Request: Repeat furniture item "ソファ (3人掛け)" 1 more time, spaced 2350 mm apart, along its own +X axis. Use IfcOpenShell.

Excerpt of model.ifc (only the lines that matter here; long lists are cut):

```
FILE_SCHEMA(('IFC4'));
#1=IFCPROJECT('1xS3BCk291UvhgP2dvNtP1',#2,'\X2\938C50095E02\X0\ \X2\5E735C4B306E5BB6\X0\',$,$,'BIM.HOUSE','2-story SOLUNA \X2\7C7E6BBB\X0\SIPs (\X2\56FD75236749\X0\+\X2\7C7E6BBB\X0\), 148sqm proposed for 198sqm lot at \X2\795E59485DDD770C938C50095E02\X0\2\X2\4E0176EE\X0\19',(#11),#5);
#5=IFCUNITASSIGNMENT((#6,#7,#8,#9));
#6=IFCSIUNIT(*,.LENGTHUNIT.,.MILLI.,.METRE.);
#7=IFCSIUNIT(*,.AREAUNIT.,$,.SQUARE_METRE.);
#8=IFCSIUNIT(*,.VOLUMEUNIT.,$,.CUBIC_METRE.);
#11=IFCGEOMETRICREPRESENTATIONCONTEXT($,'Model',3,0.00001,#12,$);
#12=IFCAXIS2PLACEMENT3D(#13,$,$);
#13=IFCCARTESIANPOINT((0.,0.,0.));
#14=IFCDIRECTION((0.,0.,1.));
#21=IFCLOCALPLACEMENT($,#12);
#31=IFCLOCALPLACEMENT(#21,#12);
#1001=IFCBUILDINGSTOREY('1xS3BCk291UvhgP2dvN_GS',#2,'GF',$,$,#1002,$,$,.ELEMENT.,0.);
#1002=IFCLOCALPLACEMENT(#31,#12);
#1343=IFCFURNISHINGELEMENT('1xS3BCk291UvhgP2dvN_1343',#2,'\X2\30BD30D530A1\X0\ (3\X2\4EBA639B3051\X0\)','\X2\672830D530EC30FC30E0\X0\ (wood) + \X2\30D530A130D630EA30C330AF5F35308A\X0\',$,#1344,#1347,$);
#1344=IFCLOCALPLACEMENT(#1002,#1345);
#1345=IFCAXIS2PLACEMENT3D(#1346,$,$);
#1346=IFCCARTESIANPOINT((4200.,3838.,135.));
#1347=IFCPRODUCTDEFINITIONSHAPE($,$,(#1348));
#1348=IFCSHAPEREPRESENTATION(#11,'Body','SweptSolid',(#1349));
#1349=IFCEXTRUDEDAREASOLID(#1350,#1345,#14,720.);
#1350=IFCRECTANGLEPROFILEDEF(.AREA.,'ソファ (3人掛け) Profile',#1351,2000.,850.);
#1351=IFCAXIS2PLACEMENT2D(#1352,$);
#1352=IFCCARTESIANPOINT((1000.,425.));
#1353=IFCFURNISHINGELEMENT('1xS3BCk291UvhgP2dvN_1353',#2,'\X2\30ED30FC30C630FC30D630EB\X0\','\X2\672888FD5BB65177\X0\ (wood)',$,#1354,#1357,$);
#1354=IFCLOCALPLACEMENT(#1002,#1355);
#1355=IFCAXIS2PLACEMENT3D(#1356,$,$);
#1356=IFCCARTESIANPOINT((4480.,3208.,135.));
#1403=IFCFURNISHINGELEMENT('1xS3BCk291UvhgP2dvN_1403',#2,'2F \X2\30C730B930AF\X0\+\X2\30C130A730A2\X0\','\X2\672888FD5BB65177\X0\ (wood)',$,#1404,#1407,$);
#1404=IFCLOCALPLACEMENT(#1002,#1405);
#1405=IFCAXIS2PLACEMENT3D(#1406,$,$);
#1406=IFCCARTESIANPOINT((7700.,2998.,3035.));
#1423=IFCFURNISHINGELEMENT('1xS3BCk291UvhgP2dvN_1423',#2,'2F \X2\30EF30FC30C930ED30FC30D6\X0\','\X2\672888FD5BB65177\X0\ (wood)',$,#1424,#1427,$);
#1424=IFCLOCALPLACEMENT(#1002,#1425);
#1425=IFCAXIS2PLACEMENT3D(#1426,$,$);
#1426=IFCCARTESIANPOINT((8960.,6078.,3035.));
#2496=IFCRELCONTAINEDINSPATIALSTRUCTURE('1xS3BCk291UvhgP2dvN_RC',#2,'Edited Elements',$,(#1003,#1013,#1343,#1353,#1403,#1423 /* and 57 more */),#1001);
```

```python
import ifcopenshell
import ifcopenshell.api.geometry
import ifcopenshell.api.root
import ifcopenshell.util.element
import ifcopenshell.util.placement
import ifcopenshell.util.unit

model = ifcopenshell.open("model.ifc")
unit_scale = ifcopenshell.util.unit.calculate_unit_scale(model)


def reuse_history(source, copy):
    """copy_class also copies each property set's owner history, people and application; keep the originals."""
    for rel in copy.IsDefinedBy:
        if rel.is_a("IfcRelDefinesByProperties") and (history := rel.RelatingPropertyDefinition.OwnerHistory):
            rel.RelatingPropertyDefinition.OwnerHistory = source.OwnerHistory
            ifcopenshell.util.element.remove_deep2(model, history)


source = model.by_guid("1xS3BCk291UvhgP2dvN_1343")
base = ifcopenshell.util.placement.get_local_placement(source.ObjectPlacement)
step = base[:3, 0] * 2.35 / unit_scale

for i in range(1, 2):
    copy = ifcopenshell.api.root.copy_class(model, product=source)
    copy.Representation = ifcopenshell.util.element.copy_deep(
        model, source.Representation, exclude=["IfcGeometricRepresentationContext", "IfcRepresentationMap"]
    )
    reuse_history(source, copy)
    matrix = base.copy()
    matrix[:3, 3] += i * step
    print("added at", matrix[:3, 3].round(3) + 0.0)
    ifcopenshell.api.geometry.edit_object_placement(model, product=copy, matrix=matrix, is_si=False)

model.write("model_v2.ifc")
```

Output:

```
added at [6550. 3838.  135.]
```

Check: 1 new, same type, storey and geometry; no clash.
